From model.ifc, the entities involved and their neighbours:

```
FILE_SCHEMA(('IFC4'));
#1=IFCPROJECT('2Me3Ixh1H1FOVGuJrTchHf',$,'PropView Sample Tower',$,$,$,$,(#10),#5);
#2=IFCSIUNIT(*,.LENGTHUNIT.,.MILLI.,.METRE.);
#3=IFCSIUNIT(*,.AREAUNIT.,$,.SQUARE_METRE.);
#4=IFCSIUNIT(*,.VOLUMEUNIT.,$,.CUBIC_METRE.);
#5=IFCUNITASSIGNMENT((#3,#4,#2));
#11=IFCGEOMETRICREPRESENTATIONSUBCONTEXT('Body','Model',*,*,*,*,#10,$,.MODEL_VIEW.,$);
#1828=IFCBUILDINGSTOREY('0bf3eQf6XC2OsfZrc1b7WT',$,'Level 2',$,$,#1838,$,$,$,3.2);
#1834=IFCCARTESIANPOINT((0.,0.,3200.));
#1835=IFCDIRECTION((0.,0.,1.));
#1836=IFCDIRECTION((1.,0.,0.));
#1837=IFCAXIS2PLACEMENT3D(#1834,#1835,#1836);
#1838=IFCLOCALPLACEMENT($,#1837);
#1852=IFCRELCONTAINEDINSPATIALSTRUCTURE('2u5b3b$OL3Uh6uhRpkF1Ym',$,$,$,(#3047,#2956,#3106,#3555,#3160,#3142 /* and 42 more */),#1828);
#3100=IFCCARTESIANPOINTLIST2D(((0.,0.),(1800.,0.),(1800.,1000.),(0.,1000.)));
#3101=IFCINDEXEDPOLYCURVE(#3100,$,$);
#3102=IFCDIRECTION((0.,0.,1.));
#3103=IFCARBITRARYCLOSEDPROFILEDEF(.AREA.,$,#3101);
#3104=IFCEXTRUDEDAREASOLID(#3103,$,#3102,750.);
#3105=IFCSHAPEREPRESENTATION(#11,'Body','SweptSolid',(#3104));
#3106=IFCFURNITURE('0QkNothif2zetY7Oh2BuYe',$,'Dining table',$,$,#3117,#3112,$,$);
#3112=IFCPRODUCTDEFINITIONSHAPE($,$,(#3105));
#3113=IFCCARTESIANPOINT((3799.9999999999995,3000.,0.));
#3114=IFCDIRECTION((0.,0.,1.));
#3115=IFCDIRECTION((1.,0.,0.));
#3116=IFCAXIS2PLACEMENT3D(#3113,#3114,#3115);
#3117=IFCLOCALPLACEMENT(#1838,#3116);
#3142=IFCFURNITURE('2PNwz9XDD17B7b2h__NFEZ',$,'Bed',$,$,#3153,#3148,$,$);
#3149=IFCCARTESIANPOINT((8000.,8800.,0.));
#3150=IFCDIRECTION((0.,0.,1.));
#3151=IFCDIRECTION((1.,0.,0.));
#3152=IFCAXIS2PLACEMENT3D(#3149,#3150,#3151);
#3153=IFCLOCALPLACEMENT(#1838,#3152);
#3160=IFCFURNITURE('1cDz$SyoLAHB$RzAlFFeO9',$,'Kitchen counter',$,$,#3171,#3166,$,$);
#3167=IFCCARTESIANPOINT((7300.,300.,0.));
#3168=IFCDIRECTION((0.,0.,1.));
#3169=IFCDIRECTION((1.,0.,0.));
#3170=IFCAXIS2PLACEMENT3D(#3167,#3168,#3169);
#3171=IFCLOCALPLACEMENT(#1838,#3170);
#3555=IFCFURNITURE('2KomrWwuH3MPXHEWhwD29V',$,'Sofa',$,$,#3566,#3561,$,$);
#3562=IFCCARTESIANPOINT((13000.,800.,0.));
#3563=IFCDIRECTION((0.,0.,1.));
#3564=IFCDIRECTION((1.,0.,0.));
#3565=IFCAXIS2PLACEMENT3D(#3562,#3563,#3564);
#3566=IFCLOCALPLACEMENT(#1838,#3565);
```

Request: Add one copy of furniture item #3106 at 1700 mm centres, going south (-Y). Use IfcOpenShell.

```python
import numpy as np
import ifcopenshell
import ifcopenshell.api.geometry
import ifcopenshell.api.root
import ifcopenshell.util.element
import ifcopenshell.util.placement
import ifcopenshell.util.unit

model = ifcopenshell.open("model.ifc")
unit_scale = ifcopenshell.util.unit.calculate_unit_scale(model)

source = model.by_guid("0QkNothif2zetY7Oh2BuYe")
base = ifcopenshell.util.placement.get_local_placement(source.ObjectPlacement)
step = np.array([0.0, -1.0, 0.0]) * 1.7 / unit_scale

for i in range(1, 2):
    copy = ifcopenshell.api.root.copy_class(model, product=source)
    copy.Representation = ifcopenshell.util.element.copy_deep(
        model, source.Representation, exclude=["IfcGeometricRepresentationContext", "IfcRepresentationMap"]
    )
    matrix = base.copy()
    matrix[:3, 3] += i * step
    print("added at", matrix[:3, 3].round(3) + 0.0)
    ifcopenshell.api.geometry.edit_object_placement(model, product=copy, matrix=matrix, is_si=False)

model.write("model_rev.ifc")
```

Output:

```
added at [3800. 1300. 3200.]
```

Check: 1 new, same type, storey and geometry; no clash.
